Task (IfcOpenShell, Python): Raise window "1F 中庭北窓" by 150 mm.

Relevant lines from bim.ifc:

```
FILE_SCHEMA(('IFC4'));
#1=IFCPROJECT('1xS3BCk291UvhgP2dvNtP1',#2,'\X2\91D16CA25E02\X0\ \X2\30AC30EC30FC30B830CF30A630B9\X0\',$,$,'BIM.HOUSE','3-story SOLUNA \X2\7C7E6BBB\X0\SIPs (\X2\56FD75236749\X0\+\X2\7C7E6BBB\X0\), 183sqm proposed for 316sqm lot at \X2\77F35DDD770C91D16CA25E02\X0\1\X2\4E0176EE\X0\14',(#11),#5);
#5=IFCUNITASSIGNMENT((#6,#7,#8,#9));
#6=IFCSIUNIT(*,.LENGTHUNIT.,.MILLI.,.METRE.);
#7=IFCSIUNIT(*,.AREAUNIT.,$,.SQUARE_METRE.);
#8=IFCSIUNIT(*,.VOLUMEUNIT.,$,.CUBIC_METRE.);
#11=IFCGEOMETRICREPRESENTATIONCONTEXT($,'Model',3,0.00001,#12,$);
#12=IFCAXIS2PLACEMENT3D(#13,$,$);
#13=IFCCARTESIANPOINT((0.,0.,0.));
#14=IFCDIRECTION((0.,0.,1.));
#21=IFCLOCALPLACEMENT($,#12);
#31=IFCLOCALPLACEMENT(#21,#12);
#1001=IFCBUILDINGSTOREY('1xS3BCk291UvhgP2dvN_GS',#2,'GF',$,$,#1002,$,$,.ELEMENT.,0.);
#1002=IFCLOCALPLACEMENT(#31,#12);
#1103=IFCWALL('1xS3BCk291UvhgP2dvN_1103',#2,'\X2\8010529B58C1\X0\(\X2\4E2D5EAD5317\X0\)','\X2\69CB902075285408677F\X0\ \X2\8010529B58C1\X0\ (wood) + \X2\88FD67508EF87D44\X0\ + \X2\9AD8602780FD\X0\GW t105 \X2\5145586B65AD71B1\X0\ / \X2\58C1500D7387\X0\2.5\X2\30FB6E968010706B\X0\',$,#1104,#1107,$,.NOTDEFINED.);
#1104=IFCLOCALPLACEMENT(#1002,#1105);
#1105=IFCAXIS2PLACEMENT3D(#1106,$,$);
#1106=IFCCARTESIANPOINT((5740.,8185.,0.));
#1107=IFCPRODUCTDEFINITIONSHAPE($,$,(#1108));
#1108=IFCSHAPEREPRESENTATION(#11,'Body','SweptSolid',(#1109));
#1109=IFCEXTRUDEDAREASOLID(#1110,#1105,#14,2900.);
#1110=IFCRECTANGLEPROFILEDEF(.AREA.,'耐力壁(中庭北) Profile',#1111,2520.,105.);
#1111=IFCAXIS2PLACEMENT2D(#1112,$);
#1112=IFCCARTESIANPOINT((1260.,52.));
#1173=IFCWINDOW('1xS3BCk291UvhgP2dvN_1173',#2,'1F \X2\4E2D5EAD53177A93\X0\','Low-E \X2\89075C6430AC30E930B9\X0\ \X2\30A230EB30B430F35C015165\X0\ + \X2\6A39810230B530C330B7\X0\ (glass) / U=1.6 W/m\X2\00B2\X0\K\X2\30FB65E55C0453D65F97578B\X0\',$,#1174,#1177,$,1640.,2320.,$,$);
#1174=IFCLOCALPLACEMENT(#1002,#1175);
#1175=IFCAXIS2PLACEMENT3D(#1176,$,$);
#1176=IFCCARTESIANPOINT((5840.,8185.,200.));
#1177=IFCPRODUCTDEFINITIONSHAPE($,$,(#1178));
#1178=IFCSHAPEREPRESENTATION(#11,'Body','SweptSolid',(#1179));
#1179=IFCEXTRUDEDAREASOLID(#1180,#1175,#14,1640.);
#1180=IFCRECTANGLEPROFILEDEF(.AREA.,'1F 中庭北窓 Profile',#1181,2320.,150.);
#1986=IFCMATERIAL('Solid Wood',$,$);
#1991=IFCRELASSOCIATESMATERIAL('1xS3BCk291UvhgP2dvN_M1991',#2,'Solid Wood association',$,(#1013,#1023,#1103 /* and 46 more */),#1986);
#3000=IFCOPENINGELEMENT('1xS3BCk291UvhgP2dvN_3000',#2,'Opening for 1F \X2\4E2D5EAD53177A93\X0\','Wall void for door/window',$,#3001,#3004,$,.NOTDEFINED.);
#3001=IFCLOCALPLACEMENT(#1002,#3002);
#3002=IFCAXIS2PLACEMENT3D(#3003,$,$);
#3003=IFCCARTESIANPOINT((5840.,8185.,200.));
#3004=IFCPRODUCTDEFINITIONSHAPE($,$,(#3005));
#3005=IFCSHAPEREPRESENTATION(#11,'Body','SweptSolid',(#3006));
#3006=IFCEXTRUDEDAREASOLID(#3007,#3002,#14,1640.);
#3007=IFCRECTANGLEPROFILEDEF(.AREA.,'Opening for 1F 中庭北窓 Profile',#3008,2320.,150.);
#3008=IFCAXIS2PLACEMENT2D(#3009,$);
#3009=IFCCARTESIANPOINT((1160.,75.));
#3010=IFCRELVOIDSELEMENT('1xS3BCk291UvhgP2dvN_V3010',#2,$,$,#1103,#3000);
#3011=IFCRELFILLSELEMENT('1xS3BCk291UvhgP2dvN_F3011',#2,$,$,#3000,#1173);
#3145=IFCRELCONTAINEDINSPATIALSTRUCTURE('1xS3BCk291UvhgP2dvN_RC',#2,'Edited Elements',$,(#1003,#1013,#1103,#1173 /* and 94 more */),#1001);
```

```python
import numpy as np
import ifcopenshell
import ifcopenshell.api.geometry
import ifcopenshell.util.placement
import ifcopenshell.util.unit

model = ifcopenshell.open("bim.ifc")
unit_scale = ifcopenshell.util.unit.calculate_unit_scale(model)

window = model.by_guid("1xS3BCk291UvhgP2dvN_1173")
opening = window.FillsVoids[0].RelatingOpeningElement
dz = 0.15 / unit_scale

shift = np.array([0.0, 0.0, dz])
# The window is not placed relative to its opening, so move both.
for product in (opening, window):
    matrix = ifcopenshell.util.placement.get_local_placement(product.ObjectPlacement)
    matrix[:3, 3] += shift
    ifcopenshell.api.geometry.edit_object_placement(model, product=product, matrix=matrix, is_si=False)

print(f"moved by {dz * unit_scale:+.3f} m")

model.write("bim_edited.ifc")
```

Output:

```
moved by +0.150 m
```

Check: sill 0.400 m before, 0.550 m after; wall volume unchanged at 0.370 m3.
